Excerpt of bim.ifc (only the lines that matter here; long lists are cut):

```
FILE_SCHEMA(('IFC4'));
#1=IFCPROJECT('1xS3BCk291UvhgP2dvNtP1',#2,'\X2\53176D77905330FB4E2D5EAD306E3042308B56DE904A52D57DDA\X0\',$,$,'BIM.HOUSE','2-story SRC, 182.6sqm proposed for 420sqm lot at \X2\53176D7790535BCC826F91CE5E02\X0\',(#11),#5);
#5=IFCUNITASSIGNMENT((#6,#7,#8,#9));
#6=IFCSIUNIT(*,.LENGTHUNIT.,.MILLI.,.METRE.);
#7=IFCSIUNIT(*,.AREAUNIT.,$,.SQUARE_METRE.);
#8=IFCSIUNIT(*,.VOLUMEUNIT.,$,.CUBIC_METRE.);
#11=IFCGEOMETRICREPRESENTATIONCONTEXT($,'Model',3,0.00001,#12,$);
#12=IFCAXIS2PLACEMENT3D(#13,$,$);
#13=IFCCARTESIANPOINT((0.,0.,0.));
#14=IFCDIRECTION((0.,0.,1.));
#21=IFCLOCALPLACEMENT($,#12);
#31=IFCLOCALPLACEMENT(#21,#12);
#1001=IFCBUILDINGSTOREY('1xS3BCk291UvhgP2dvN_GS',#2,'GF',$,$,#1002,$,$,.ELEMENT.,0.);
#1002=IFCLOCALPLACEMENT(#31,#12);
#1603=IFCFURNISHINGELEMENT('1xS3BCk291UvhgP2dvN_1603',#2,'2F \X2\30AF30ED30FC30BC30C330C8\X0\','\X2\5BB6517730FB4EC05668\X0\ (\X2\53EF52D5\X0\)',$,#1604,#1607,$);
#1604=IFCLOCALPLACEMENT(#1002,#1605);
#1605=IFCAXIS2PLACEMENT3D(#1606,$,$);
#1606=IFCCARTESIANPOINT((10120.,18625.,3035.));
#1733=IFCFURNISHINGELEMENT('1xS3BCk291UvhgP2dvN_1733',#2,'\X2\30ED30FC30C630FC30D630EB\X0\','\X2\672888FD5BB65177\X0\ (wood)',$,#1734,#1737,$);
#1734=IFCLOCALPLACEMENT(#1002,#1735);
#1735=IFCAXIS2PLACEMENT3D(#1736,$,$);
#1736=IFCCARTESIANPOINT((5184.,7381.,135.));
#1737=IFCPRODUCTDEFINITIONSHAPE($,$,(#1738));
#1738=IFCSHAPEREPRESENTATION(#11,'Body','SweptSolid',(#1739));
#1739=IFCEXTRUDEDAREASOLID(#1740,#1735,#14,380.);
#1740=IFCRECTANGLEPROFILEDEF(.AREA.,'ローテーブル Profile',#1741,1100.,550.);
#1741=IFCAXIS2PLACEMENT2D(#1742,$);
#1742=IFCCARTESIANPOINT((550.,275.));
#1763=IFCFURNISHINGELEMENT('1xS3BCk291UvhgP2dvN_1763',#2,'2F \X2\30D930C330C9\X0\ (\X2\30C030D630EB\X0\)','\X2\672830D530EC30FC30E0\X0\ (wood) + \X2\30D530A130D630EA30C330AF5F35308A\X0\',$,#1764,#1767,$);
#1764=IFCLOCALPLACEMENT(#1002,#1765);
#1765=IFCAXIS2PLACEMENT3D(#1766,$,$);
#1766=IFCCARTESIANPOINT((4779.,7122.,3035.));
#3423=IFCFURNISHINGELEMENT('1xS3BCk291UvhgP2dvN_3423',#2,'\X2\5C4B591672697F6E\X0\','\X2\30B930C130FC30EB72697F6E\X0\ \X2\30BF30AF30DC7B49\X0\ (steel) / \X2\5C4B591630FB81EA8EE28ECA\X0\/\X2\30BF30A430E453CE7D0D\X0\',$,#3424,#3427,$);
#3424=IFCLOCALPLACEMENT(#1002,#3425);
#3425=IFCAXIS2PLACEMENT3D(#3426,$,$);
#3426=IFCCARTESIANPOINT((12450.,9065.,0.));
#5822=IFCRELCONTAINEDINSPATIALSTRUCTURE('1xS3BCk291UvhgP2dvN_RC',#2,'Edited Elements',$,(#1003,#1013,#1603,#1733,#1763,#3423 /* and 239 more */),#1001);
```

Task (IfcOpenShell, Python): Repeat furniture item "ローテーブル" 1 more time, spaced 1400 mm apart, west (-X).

```python
import numpy as np
import ifcopenshell
import ifcopenshell.api.geometry
import ifcopenshell.api.root
import ifcopenshell.util.element
import ifcopenshell.util.placement

model = ifcopenshell.open("bim.ifc")


def reuse_history(source, copy):
    """copy_class also copies each property set's owner history, people and application; keep the originals."""
    for rel in copy.IsDefinedBy:
        if rel.is_a("IfcRelDefinesByProperties") and (history := rel.RelatingPropertyDefinition.OwnerHistory):
            rel.RelatingPropertyDefinition.OwnerHistory = source.OwnerHistory
            ifcopenshell.util.element.remove_deep2(model, history)


source = model.by_id(1733)
base = ifcopenshell.util.placement.get_local_placement(source.ObjectPlacement)
step = np.array([-1.0, 0.0, 0.0]) * 1400.0

for i in range(1, 2):
    copy = ifcopenshell.api.root.copy_class(model, product=source)
    copy.Representation = ifcopenshell.util.element.copy_deep(
        model, source.Representation, exclude=["IfcGeometricRepresentationContext", "IfcRepresentationMap"]
    )
    reuse_history(source, copy)
    matrix = base.copy()
    matrix[:3, 3] += i * step
    print("added at", matrix[:3, 3].round(3) + 0.0)
    ifcopenshell.api.geometry.edit_object_placement(model, product=copy, matrix=matrix, is_si=False)

model.write("bim_edited.ifc")
```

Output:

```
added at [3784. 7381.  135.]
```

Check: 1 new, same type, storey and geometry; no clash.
